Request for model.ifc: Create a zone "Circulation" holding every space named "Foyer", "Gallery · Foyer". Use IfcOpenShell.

First a look at what the model holds.

```python
import ifcopenshell

model = ifcopenshell.open("model.ifc")
print(model.schema)
seen = {}
for space in model.by_type("IfcSpace"):
    seen[space.Name] = seen.get(space.Name, 0) + 1
for name, count in sorted(seen.items(), key=str):
    print(count, "x", name)
print("zones:", [z.Name for z in model.by_type("IfcZone")][:20])
```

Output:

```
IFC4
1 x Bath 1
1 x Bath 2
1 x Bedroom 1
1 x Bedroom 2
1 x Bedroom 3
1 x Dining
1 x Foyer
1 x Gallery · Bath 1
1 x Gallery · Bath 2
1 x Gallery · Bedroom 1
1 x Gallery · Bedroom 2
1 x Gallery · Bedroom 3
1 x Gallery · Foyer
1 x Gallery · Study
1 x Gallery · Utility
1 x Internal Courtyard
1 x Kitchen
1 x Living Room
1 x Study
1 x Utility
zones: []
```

```python
import ifcopenshell
import ifcopenshell.api.group
import ifcopenshell.api.root

model = ifcopenshell.open("model.ifc")

names = {"Foyer", "Gallery · Foyer"}
spaces = [s for s in model.by_type("IfcSpace") if s.Name in names]

zone = ifcopenshell.api.root.create_entity(model, ifc_class="IfcZone", name="Circulation")
ifcopenshell.api.group.assign_group(model, products=spaces, group=zone)
print(len(spaces), "spaces in", zone.Name)

model.write("model_rev.ifc")
```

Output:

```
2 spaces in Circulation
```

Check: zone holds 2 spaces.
